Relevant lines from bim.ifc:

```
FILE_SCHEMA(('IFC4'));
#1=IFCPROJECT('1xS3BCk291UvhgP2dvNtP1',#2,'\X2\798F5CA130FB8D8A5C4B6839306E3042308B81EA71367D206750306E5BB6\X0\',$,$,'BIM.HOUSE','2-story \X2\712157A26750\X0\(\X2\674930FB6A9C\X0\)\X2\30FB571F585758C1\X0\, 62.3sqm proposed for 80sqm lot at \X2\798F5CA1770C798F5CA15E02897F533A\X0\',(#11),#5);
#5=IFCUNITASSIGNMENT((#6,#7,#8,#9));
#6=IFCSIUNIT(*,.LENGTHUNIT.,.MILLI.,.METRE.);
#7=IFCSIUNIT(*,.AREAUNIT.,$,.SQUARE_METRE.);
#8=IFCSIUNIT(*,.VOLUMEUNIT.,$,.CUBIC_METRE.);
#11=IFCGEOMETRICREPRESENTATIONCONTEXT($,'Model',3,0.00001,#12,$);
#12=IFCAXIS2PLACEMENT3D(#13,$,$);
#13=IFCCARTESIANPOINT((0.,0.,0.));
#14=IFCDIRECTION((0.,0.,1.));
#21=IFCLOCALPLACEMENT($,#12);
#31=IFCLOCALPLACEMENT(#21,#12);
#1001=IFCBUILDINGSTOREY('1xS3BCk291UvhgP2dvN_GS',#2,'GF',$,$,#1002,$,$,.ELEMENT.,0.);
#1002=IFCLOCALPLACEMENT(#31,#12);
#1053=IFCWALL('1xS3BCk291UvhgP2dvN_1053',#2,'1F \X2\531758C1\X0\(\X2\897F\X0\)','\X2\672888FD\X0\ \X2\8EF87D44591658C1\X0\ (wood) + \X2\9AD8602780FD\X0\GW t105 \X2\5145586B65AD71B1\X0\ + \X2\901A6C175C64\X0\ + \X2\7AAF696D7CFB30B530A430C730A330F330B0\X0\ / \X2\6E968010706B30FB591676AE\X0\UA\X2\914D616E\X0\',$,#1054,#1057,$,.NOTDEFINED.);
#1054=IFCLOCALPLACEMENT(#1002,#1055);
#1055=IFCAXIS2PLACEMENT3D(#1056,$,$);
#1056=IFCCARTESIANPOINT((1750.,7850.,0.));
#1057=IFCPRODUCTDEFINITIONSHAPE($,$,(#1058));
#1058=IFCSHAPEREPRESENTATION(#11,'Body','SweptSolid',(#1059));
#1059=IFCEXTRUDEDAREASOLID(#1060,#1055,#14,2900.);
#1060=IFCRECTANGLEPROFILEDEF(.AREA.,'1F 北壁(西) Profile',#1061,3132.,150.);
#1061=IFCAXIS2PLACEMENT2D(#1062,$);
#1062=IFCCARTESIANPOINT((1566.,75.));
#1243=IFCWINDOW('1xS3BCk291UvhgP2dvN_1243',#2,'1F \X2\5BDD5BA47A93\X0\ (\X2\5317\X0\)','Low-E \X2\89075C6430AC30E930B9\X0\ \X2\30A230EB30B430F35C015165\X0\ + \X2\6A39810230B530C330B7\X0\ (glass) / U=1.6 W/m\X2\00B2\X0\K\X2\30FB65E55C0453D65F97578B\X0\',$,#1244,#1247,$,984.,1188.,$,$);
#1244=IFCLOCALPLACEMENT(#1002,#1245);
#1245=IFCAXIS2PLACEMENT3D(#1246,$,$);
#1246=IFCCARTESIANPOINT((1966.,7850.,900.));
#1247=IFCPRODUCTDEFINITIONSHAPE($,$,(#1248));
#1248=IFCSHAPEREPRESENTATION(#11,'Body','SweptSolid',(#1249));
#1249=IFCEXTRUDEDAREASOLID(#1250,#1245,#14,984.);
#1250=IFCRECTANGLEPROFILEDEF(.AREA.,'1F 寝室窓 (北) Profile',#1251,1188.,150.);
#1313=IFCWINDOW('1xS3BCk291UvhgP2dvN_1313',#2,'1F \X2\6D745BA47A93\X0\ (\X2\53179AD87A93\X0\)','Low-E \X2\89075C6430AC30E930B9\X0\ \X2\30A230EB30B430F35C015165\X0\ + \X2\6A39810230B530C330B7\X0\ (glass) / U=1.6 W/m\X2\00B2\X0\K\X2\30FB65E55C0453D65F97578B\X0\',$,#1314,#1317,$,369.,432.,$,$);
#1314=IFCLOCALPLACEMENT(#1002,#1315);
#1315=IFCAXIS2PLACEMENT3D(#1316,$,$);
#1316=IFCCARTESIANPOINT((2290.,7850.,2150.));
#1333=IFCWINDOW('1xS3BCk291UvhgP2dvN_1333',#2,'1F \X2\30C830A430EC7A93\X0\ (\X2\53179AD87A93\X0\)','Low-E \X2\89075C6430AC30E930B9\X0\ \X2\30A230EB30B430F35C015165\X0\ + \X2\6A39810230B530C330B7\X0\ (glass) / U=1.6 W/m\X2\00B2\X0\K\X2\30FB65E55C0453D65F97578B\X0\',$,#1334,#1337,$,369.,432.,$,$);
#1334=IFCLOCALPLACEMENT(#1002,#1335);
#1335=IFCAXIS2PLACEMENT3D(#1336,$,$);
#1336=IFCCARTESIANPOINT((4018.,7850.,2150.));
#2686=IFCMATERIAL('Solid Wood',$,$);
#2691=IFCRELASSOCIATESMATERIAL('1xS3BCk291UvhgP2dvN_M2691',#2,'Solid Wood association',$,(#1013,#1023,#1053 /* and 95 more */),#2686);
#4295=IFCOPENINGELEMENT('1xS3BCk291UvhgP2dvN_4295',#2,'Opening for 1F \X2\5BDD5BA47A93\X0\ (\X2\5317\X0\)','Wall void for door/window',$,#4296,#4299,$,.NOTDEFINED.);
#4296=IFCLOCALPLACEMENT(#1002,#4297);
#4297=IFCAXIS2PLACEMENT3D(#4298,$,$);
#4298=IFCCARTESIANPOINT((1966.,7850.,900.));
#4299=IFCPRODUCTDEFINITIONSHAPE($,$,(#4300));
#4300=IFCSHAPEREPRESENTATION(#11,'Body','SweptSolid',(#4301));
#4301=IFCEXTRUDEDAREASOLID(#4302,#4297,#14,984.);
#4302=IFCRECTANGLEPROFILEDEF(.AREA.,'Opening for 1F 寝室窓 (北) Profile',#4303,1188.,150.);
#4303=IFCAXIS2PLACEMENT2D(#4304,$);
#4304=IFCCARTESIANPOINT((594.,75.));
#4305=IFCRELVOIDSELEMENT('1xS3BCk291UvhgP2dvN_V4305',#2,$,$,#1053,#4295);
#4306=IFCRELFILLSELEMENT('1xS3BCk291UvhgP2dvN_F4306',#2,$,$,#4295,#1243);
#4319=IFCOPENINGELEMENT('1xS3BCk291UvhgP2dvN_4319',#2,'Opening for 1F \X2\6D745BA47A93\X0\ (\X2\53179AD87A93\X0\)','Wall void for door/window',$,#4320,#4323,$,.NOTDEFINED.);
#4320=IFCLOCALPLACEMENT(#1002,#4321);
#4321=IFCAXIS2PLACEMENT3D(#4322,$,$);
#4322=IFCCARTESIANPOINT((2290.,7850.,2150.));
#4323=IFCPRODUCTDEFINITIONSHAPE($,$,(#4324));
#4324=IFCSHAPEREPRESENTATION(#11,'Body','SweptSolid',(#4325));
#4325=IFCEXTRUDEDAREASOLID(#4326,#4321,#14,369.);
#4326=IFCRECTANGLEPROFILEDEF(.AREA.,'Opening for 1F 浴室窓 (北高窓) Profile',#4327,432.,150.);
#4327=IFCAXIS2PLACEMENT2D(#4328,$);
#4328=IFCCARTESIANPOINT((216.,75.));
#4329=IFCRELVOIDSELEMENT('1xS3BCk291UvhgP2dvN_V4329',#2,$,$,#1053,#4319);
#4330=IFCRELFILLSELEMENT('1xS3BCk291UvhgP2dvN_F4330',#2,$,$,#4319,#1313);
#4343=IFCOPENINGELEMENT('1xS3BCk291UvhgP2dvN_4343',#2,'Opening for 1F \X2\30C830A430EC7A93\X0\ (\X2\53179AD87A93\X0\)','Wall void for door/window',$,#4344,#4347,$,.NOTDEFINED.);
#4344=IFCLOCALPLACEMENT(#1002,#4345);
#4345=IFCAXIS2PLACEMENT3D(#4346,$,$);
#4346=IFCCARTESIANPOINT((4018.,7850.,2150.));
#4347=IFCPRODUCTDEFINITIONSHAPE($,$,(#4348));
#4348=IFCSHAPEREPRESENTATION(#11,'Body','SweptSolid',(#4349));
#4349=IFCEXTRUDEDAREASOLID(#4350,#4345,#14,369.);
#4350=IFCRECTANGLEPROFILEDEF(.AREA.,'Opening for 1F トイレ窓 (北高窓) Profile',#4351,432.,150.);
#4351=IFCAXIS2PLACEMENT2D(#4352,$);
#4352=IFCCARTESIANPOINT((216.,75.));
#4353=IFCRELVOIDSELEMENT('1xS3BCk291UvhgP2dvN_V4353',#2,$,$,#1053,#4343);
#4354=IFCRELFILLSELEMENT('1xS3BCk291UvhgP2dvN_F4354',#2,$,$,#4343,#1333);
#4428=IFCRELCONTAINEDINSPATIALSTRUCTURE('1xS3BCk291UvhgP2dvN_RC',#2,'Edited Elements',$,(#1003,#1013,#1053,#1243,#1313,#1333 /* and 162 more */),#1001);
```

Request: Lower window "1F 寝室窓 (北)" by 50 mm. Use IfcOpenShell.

```python
import numpy as np
import ifcopenshell
import ifcopenshell.api.geometry
import ifcopenshell.util.placement
import ifcopenshell.util.unit

model = ifcopenshell.open("bim.ifc")
unit_scale = ifcopenshell.util.unit.calculate_unit_scale(model)

window = model.by_guid("1xS3BCk291UvhgP2dvN_1243")
opening = window.FillsVoids[0].RelatingOpeningElement
dz = -0.05 / unit_scale

shift = np.array([0.0, 0.0, dz])
# The window is not placed relative to its opening, so move both.
for product in (opening, window):
    matrix = ifcopenshell.util.placement.get_local_placement(product.ObjectPlacement)
    matrix[:3, 3] += shift
    ifcopenshell.api.geometry.edit_object_placement(model, product=product, matrix=matrix, is_si=False)

print(f"moved by {dz * unit_scale:+.3f} m")

model.write("bim_rev.ifc")
```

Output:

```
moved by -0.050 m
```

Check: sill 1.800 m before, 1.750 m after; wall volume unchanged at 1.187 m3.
